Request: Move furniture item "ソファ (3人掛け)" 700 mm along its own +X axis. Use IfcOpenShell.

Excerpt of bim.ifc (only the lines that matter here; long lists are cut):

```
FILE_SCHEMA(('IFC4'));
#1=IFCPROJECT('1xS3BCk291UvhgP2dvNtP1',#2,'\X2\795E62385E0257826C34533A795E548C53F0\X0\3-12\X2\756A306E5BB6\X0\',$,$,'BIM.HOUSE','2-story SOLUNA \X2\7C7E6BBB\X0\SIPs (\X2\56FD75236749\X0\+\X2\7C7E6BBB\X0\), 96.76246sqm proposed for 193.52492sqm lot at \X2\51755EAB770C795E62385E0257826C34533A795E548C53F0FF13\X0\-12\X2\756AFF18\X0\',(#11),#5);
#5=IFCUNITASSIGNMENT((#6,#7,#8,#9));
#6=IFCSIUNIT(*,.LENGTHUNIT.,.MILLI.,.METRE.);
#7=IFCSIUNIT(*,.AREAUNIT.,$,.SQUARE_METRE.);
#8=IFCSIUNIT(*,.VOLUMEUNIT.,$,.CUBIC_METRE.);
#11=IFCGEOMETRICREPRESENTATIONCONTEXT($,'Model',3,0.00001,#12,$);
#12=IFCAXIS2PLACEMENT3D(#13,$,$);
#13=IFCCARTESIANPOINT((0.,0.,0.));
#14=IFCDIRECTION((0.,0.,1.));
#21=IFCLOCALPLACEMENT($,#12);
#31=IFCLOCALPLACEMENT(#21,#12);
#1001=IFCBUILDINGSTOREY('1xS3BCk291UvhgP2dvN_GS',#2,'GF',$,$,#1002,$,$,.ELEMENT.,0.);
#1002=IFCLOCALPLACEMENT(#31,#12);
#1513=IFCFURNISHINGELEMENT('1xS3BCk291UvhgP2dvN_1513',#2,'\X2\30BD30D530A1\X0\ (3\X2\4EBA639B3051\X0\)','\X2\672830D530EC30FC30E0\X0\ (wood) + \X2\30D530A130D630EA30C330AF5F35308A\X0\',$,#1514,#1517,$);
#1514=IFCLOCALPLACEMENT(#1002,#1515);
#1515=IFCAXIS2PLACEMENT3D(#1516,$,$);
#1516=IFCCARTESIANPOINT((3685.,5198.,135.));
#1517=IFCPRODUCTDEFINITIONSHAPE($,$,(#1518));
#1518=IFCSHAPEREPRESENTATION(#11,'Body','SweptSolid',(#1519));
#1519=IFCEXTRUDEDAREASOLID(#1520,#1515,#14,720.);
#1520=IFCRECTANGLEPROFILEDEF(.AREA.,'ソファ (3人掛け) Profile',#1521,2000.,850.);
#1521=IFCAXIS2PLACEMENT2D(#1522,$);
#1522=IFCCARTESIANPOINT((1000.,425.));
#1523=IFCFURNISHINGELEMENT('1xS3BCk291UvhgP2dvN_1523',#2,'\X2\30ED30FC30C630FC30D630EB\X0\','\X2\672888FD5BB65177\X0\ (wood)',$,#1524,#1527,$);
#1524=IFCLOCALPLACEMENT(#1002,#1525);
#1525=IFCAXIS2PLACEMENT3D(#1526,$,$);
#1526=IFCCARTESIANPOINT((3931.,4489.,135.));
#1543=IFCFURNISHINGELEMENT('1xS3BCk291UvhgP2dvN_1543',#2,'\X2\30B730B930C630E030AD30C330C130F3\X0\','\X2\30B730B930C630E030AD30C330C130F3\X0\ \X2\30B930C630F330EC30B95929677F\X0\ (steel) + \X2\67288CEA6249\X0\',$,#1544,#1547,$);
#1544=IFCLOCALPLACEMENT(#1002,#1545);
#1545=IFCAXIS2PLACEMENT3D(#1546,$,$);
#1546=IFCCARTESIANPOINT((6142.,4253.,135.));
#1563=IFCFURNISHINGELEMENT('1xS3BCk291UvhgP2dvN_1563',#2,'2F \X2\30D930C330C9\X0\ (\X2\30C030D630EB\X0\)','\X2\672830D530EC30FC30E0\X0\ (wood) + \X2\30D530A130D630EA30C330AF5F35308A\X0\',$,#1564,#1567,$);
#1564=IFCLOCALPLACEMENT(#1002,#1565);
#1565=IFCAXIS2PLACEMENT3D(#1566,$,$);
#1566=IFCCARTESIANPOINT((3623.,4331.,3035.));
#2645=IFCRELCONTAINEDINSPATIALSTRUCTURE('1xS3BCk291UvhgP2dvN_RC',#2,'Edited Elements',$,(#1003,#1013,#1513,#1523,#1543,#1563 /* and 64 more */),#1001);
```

```python
import ifcopenshell
import ifcopenshell.api.geometry
import ifcopenshell.util.placement

model = ifcopenshell.open("bim.ifc")

item = model.by_id(1513)
matrix = ifcopenshell.util.placement.get_local_placement(item.ObjectPlacement)
matrix[:3, 3] += matrix[:3, 0] * 700.0
ifcopenshell.api.geometry.edit_object_placement(model, product=item, matrix=matrix, is_si=False)

print(ifcopenshell.util.placement.get_local_placement(item.ObjectPlacement).round(3) + 0.0)

model.write("bim_edited.ifc")
```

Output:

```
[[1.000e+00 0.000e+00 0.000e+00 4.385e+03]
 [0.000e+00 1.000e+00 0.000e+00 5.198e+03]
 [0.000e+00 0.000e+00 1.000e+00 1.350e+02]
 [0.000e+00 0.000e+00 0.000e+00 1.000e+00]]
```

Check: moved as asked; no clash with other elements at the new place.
